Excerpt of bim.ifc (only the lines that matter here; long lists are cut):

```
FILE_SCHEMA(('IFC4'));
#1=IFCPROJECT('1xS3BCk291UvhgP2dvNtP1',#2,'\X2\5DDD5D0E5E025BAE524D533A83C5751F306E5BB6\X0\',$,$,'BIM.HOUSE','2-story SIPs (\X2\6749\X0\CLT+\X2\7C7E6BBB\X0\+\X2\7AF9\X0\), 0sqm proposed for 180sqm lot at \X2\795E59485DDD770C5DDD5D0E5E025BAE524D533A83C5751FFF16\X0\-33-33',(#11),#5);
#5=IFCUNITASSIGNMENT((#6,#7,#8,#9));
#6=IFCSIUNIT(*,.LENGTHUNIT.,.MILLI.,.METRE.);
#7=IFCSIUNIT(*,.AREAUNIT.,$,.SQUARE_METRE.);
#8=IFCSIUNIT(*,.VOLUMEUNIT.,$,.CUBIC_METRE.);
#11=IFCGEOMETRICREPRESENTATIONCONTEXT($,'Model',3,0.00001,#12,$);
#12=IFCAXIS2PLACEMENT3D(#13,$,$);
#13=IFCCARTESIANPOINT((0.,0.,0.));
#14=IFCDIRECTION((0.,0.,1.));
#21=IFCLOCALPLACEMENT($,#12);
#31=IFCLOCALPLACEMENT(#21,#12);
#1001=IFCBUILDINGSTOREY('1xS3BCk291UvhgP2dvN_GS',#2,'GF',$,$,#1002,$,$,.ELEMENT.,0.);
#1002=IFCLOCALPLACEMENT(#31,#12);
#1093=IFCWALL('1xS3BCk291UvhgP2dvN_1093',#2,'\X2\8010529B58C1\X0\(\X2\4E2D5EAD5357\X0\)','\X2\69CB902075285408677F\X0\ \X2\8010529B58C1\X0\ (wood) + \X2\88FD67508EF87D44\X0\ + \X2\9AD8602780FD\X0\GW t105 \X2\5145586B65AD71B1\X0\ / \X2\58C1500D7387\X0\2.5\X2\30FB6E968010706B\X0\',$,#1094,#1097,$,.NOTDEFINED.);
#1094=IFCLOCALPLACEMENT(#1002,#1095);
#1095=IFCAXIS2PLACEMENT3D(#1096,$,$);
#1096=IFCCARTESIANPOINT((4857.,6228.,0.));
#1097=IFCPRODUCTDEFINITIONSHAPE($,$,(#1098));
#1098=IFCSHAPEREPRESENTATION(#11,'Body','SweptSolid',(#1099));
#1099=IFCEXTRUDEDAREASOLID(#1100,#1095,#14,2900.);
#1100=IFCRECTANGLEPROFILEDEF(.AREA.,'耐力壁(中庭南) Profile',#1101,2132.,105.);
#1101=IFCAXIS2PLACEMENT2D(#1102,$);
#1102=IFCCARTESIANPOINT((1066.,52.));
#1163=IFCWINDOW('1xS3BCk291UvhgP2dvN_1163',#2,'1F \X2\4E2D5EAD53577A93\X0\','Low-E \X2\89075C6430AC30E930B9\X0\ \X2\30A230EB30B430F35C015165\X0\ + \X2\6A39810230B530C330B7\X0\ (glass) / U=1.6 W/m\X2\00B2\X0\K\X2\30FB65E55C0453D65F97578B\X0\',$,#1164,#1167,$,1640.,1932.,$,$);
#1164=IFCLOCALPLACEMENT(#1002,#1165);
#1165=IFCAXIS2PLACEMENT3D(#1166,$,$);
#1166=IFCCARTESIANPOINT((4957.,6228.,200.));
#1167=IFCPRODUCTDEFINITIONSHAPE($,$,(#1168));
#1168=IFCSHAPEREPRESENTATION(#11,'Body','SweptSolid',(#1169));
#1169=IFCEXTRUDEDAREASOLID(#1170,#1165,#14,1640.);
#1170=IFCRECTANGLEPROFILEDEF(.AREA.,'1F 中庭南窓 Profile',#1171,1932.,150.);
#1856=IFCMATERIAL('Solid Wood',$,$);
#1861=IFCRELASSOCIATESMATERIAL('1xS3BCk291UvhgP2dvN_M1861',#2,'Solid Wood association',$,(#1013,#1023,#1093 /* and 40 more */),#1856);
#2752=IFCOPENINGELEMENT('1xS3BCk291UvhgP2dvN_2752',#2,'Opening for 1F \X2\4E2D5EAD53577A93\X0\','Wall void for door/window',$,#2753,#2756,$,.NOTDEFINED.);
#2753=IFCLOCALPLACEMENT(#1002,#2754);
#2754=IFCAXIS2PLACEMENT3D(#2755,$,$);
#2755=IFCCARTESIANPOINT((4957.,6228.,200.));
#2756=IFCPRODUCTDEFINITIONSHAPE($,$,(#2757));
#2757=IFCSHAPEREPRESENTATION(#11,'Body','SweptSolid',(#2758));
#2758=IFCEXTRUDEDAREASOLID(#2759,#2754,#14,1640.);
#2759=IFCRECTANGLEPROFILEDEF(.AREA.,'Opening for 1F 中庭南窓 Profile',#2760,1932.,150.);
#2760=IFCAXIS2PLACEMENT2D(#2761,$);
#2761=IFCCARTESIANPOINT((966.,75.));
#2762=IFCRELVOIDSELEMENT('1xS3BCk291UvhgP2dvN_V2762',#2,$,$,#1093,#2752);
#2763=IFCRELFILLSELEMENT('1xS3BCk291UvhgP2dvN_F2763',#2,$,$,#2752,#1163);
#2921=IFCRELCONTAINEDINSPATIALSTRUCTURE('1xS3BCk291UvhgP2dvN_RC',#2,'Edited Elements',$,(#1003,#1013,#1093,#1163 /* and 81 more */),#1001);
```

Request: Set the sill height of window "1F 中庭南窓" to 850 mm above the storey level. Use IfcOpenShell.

```python
import numpy as np
import ifcopenshell
import ifcopenshell.api.geometry
import ifcopenshell.geom
import ifcopenshell.util.element
import ifcopenshell.util.placement
import ifcopenshell.util.shape
import ifcopenshell.util.unit

model = ifcopenshell.open("bim.ifc")
unit_scale = ifcopenshell.util.unit.calculate_unit_scale(model)

window = model.by_guid("1xS3BCk291UvhgP2dvN_1163")
opening = window.FillsVoids[0].RelatingOpeningElement
storey = ifcopenshell.util.element.get_container(window, ifc_class="IfcBuildingStorey")
level = ifcopenshell.util.placement.get_local_placement(storey.ObjectPlacement)[2, 3]

# The opening's origin need not be at the sill, so measure its lowest point.
shape = ifcopenshell.geom.create_shape(ifcopenshell.geom.settings(), opening)
bottom = ifcopenshell.util.shape.get_shape_bottom_elevation(shape, shape.geometry) / unit_scale
dz = level + 850.0 - bottom

shift = np.array([0.0, 0.0, dz])
# The window is not placed relative to its opening, so move both.
for product in (opening, window):
    matrix = ifcopenshell.util.placement.get_local_placement(product.ObjectPlacement)
    matrix[:3, 3] += shift
    ifcopenshell.api.geometry.edit_object_placement(model, product=product, matrix=matrix, is_si=False)

print(f"moved by {dz * unit_scale:+.3f} m")

model.write("bim_rev.ifc")
```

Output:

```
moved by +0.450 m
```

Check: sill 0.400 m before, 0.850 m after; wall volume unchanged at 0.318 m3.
